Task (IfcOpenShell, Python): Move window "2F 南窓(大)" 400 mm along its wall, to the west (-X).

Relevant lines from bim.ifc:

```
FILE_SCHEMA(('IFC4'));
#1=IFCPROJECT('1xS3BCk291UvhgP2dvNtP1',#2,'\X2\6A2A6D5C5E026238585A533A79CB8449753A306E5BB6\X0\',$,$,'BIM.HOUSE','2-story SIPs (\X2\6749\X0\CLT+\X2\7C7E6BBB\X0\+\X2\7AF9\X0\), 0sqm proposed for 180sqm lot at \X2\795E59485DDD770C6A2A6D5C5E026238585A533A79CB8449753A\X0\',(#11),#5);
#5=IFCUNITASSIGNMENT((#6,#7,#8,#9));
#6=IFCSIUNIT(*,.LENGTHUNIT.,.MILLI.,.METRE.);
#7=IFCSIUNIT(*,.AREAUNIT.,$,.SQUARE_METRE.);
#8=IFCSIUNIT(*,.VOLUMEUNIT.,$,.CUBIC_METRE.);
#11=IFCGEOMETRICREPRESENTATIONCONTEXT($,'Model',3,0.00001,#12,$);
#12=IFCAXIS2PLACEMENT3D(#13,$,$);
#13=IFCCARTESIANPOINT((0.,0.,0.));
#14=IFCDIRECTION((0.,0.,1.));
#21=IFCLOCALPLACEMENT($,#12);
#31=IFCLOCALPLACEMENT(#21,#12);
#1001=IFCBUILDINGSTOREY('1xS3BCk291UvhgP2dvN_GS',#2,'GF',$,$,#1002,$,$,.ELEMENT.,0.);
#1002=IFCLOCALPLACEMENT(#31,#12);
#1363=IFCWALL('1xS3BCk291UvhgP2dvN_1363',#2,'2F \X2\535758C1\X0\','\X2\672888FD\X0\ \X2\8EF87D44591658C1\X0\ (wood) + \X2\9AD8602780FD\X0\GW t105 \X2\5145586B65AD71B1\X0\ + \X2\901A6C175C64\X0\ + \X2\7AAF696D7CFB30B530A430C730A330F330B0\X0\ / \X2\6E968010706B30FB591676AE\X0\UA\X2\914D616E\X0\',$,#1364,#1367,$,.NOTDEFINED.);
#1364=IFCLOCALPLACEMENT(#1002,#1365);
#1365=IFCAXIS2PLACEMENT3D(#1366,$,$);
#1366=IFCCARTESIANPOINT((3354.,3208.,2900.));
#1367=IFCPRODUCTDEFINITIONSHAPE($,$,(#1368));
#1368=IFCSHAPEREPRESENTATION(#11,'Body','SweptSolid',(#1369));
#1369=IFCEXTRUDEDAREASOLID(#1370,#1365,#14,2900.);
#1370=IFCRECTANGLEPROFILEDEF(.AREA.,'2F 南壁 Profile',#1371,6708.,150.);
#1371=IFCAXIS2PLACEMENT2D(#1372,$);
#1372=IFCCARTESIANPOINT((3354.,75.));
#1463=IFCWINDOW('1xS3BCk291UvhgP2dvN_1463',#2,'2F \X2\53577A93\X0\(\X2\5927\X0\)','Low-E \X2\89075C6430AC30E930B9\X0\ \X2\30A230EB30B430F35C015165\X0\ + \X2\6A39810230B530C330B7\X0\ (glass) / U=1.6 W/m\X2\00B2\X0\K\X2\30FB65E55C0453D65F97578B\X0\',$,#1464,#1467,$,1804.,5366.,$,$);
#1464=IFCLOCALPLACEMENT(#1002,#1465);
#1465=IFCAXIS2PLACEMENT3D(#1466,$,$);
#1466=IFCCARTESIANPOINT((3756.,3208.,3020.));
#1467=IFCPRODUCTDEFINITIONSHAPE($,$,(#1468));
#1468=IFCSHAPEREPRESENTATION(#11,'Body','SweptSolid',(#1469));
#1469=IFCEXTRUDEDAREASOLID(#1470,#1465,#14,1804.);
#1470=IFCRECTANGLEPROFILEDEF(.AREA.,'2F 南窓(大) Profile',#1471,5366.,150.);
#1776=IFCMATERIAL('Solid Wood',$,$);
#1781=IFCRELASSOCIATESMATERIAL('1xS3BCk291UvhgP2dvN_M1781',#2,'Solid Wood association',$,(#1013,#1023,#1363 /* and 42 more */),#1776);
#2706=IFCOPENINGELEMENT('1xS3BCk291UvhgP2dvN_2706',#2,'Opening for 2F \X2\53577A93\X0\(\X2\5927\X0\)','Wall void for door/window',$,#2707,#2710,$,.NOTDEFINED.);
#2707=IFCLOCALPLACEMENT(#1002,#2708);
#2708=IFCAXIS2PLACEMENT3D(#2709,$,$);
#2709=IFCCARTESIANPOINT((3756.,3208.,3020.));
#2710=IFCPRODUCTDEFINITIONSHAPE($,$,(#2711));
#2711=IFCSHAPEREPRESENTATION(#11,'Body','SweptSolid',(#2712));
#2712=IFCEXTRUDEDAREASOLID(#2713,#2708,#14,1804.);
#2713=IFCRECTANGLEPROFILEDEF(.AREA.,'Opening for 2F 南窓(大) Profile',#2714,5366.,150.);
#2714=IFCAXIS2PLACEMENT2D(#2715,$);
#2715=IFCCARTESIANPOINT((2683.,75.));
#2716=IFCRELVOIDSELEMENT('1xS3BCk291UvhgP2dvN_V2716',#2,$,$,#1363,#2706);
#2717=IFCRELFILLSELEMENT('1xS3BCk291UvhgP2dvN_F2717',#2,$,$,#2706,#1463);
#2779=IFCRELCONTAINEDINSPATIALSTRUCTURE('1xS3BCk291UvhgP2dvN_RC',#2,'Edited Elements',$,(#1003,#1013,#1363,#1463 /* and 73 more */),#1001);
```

```python
import ifcopenshell
import ifcopenshell.api.geometry
import ifcopenshell.util.placement
import ifcopenshell.util.unit

model = ifcopenshell.open("bim.ifc")
unit_scale = ifcopenshell.util.unit.calculate_unit_scale(model)

window = model.by_guid("1xS3BCk291UvhgP2dvN_1463")
opening = window.FillsVoids[0].RelatingOpeningElement
wall = opening.VoidsElements[0].RelatingBuildingElement

wall_matrix = ifcopenshell.util.placement.get_local_placement(wall.ObjectPlacement)
shift = wall_matrix[:3, 0] * -0.4 / unit_scale
before = ifcopenshell.util.placement.get_local_placement(window.ObjectPlacement)[:3, 3].copy()

# The window is not placed relative to its opening, so move both.
for product in (opening, window):
    matrix = ifcopenshell.util.placement.get_local_placement(product.ObjectPlacement)
    matrix[:3, 3] += shift
    ifcopenshell.api.geometry.edit_object_placement(model, product=product, matrix=matrix, is_si=False)

after = ifcopenshell.util.placement.get_local_placement(window.ObjectPlacement)[:3, 3]
print("window moved by", (after - before).round(3) + 0.0)

model.write("bim_edited.ifc")
```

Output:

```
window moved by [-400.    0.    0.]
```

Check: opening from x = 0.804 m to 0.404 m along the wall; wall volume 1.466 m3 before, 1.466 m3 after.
